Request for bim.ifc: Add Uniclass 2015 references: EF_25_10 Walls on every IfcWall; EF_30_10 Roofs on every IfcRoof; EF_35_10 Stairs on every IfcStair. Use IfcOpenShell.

First a look at what the model holds.

```python
import ifcopenshell

model = ifcopenshell.open("bim.ifc")
print(model.schema)
print("classifications:", [c.Name for c in model.by_type("IfcClassification")])
for ifc_class in ("IfcDoor", "IfcRoof", "IfcStair", "IfcWall", "IfcWindow"):
    print(ifc_class, len(model.by_type(ifc_class)))
```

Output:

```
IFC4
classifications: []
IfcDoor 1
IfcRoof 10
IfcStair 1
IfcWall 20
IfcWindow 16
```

```python
import ifcopenshell
import ifcopenshell.api.classification

model = ifcopenshell.open("bim.ifc")

system = ifcopenshell.api.classification.add_classification(model, classification="Uniclass 2015")

codes = {
    "IfcWall": ("EF_25_10", "Walls"),
    "IfcRoof": ("EF_30_10", "Roofs"),
    "IfcStair": ("EF_35_10", "Stairs"),
}
for ifc_class, (code, name) in codes.items():
    products = model.by_type(ifc_class)
    ifcopenshell.api.classification.add_reference(
        model, products=products, classification=system, identification=code, name=name
    )
    print(code, len(products))

model.write("bim_edited.ifc")
```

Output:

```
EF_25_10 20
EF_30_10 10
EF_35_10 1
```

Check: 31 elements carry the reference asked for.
